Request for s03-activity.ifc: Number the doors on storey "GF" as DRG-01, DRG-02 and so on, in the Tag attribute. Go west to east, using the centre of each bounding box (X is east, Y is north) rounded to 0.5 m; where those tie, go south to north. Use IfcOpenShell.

First a look at what the model holds.

```python
import ifcopenshell
import ifcopenshell.util.element
import ifcopenshell.util.placement

model = ifcopenshell.open("s03-activity.ifc")
print(model.schema)
storey = next(s for s in model.by_type("IfcBuildingStorey") if s.Name == "GF")
doors = [e for e in ifcopenshell.util.element.get_decomposition(storey) if e.is_a("IfcDoor")]
for e in sorted(doors, key=lambda e: e.id()):
    origin = ifcopenshell.util.placement.get_local_placement(e.ObjectPlacement)[:3, 3]
    print(e.id(), e.Tag, e.Name, origin.round(2) + 0.0, sep=" | ")
```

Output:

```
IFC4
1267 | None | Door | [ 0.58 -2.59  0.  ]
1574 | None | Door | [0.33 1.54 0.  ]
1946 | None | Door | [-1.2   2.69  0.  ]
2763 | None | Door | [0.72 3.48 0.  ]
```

```python
import ifcopenshell
import ifcopenshell.geom
import ifcopenshell.util.element
import ifcopenshell.util.shape

model = ifcopenshell.open("s03-activity.ifc")
settings = ifcopenshell.geom.settings()
settings.set("use-world-coords", True)


def centre(element):
    shape = ifcopenshell.geom.create_shape(settings, element)
    return ifcopenshell.util.shape.get_bbox_centroid(shape.geometry)


storey = next(s for s in model.by_type("IfcBuildingStorey") if s.Name == "GF")
doors = [e for e in ifcopenshell.util.element.get_decomposition(storey) if e.is_a("IfcDoor")]

# Insertion points can sit at a corner or the storey origin, so sort by the geometry (in metres).
centres = {e: centre(e) for e in doors}
doors.sort(key=lambda e: (round(centres[e][0] / 0.5), centres[e][1]))

for i, e in enumerate(doors, start=1):
    number = f"DRG-{i:02d}"
    e.Tag = number
    print(e.id(), number)

model.write("s03-activity_v2.ifc")
```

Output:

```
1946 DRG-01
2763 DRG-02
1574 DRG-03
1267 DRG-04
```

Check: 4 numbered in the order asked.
